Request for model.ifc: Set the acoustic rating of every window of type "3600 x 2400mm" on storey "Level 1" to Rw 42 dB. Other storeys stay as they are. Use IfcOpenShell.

First a look at what the model holds.

```python
import ifcopenshell
import ifcopenshell.util.element

model = ifcopenshell.open("model.ifc")
print(model.schema)
storey = next(s for s in model.by_type("IfcBuildingStorey") if s.Name == "Level 1")
windows = [e for e in ifcopenshell.util.element.get_decomposition(storey) if e.is_a("IfcWindow")]
seen = {}
for e in windows:
    element_type = ifcopenshell.util.element.get_type(e)
    key = (element_type.Name if element_type != e and element_type else None, ifcopenshell.util.element.get_pset(e, "Pset_WindowCommon", "AcousticRating"))
    seen[key] = seen.get(key, 0) + 1
for (name, value), count in sorted(seen.items(), key=str):
    print(count, "x", name, "|", value)
```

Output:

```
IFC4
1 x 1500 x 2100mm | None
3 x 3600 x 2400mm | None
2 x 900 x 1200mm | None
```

```python
import ifcopenshell
import ifcopenshell.api.pset
import ifcopenshell.util.element

model = ifcopenshell.open("model.ifc")

storey = next(s for s in model.by_type("IfcBuildingStorey") if s.Name == "Level 1")
windows = [e for e in ifcopenshell.util.element.get_decomposition(storey) if e.is_a("IfcWindow")]

count = 0
for e in windows:
    element_type = ifcopenshell.util.element.get_type(e)
    if element_type in (None, e) or element_type.Name != "3600 x 2400mm":
        continue
    # add_pset returns the element's existing set when there is one.
    pset = ifcopenshell.api.pset.add_pset(model, product=e, name="Pset_WindowCommon")
    ifcopenshell.api.pset.edit_pset(model, pset=pset, properties={"AcousticRating": "Rw 42 dB"})
    count += 1

print(count, "windows updated")

model.write("model_v2.ifc")
```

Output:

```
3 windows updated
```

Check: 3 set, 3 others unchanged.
